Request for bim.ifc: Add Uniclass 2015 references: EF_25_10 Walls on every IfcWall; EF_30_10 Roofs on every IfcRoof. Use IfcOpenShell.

First a look at what the model holds.

```python
import ifcopenshell

model = ifcopenshell.open("bim.ifc")
print(model.schema)
print("classifications:", [c.Name for c in model.by_type("IfcClassification")])
for ifc_class in ("IfcDoor", "IfcRoof", "IfcStair", "IfcWall", "IfcWindow"):
    print(ifc_class, len(model.by_type(ifc_class)))
```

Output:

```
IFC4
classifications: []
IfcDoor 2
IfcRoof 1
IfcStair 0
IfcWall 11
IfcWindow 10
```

```python
import ifcopenshell
import ifcopenshell.api.classification

model = ifcopenshell.open("bim.ifc")

system = ifcopenshell.api.classification.add_classification(model, classification="Uniclass 2015")

codes = {
    "IfcWall": ("EF_25_10", "Walls"),
    "IfcRoof": ("EF_30_10", "Roofs"),
}
for ifc_class, (code, name) in codes.items():
    products = model.by_type(ifc_class)
    ifcopenshell.api.classification.add_reference(
        model, products=products, classification=system, identification=code, name=name
    )
    print(code, len(products))

model.write("bim_edited.ifc")
```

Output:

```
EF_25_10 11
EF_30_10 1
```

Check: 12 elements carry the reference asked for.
